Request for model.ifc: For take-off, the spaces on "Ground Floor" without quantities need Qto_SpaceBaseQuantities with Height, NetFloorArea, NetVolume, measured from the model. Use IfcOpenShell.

First a look at what the model holds.

```python
import ifcopenshell
import ifcopenshell.util.element
import ifcopenshell.util.unit

model = ifcopenshell.open("model.ifc")
print(model.schema)
for unit_type in ("LENGTHUNIT", "AREAUNIT", "VOLUMEUNIT"):
    print(unit_type, ifcopenshell.util.unit.calculate_unit_scale(model, unit_type))
storey = next(s for s in model.by_type("IfcBuildingStorey") if s.Name == "Ground Floor")
spaces = [e for e in ifcopenshell.util.element.get_decomposition(storey) if e.is_a("IfcSpace")]
for e in sorted(spaces, key=lambda e: e.id()):
    print(e.id(), e.is_a(), e.Name, list(ifcopenshell.util.element.get_psets(e, qtos_only=True)), sep=" | ")
```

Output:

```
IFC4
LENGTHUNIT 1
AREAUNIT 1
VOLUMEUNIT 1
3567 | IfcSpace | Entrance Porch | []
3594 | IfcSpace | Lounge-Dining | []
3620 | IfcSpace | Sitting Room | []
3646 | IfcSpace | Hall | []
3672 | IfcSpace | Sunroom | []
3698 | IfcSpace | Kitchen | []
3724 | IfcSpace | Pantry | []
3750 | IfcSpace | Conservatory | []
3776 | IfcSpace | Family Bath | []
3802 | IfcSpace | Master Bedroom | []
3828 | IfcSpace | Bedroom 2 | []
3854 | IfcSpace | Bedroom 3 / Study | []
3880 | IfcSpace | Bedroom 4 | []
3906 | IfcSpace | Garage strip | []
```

```python
import ifcopenshell
import ifcopenshell.api.pset
import ifcopenshell.geom
import ifcopenshell.util.element
import ifcopenshell.util.shape
import ifcopenshell.util.unit

model = ifcopenshell.open("model.ifc")
unit_scale = ifcopenshell.util.unit.calculate_unit_scale(model)
area_scale = ifcopenshell.util.unit.calculate_unit_scale(model, "AREAUNIT")
volume_scale = ifcopenshell.util.unit.calculate_unit_scale(model, "VOLUMEUNIT")
settings = ifcopenshell.geom.settings()

storey = next(s for s in model.by_type("IfcBuildingStorey") if s.Name == "Ground Floor")
spaces = [e for e in ifcopenshell.util.element.get_decomposition(storey) if e.is_a("IfcSpace")]

for e in sorted(spaces, key=lambda e: e.id()):
    if ifcopenshell.util.element.get_psets(e, qtos_only=True, should_inherit=False):
        continue
    # Geometry comes back in metres, in the element's own axes.
    shape = ifcopenshell.geom.create_shape(settings, e)
    values = {
        "Height": ifcopenshell.util.shape.get_z(shape.geometry) / unit_scale,
        "NetFloorArea": ifcopenshell.util.shape.get_footprint_area(shape.geometry) / area_scale,
        "NetVolume": ifcopenshell.util.shape.get_volume(shape.geometry) / volume_scale,
    }
    qto = ifcopenshell.api.pset.add_qto(model, product=e, name="Qto_SpaceBaseQuantities")
    ifcopenshell.api.pset.edit_qto(model, qto=qto, properties=values)
    print(e.id(), {k: round(v, 3) for k, v in values.items()})

model.write("model_v2.ifc")
```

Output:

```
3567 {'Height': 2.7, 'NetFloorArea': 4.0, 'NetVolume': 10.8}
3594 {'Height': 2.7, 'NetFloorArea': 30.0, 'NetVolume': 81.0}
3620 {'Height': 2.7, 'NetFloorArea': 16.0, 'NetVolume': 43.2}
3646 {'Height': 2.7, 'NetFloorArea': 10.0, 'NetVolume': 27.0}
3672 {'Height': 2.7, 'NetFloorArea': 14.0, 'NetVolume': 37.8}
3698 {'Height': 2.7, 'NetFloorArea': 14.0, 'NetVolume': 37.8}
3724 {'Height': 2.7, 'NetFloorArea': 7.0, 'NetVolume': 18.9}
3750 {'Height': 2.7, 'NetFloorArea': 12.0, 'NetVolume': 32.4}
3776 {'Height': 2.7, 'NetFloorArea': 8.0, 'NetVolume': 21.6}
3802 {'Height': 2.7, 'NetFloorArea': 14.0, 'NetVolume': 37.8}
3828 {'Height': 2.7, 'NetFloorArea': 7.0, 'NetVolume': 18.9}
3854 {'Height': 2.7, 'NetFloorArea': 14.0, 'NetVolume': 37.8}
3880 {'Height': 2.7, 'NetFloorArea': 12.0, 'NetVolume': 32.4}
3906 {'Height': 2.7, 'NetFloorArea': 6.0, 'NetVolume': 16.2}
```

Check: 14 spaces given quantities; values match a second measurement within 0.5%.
